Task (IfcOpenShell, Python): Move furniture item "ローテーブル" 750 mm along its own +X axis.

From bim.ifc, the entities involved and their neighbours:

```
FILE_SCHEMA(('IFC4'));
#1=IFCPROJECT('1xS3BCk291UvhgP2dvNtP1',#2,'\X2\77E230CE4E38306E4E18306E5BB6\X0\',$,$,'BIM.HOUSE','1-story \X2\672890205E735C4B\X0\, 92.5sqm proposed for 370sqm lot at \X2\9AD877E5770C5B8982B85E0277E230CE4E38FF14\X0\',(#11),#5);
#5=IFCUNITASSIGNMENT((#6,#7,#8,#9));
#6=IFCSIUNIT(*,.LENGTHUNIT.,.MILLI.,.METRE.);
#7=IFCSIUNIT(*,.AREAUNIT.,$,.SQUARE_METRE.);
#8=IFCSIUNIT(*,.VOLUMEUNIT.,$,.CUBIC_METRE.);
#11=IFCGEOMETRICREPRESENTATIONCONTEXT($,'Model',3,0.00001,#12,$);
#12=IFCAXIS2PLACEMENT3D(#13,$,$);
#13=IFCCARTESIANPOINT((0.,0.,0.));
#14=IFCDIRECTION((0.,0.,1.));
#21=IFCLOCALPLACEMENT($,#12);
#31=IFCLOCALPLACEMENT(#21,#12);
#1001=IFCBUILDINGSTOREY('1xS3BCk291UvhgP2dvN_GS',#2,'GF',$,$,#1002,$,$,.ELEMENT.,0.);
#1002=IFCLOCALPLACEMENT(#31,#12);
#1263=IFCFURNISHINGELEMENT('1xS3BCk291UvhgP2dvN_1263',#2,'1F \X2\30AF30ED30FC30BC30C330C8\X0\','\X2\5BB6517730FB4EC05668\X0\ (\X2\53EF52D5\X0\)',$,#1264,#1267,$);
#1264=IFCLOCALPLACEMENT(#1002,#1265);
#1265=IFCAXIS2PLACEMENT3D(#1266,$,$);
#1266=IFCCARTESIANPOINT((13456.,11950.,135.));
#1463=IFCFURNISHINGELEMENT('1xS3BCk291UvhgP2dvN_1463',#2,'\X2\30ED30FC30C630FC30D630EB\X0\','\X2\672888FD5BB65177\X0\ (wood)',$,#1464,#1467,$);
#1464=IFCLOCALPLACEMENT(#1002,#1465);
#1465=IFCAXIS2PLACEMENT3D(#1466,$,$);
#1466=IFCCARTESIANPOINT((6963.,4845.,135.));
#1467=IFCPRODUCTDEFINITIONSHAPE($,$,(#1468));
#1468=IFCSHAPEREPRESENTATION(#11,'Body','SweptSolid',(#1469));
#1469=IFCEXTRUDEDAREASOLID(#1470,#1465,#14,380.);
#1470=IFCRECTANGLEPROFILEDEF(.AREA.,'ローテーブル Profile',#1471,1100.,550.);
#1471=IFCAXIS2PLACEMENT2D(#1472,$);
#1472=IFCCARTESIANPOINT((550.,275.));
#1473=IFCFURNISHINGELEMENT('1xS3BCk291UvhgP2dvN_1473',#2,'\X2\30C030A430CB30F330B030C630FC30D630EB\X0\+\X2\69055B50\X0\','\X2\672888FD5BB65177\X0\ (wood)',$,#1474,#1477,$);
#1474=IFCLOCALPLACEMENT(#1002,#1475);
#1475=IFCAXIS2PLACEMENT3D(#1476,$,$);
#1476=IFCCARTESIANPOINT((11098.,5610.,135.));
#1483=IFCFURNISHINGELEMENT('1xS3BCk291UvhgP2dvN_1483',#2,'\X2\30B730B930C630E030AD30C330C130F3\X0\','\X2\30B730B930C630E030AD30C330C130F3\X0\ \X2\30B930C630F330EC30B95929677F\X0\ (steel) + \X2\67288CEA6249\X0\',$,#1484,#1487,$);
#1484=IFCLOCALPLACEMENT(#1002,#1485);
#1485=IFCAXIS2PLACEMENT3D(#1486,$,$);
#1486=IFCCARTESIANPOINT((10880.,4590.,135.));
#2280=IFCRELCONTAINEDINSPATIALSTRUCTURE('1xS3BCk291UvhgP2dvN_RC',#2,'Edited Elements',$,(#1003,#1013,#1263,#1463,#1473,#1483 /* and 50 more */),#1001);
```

```python
import ifcopenshell
import ifcopenshell.api.geometry
import ifcopenshell.util.placement

model = ifcopenshell.open("bim.ifc")

item = model.by_guid("1xS3BCk291UvhgP2dvN_1463")
matrix = ifcopenshell.util.placement.get_local_placement(item.ObjectPlacement)
matrix[:3, 3] += matrix[:3, 0] * 750.0
ifcopenshell.api.geometry.edit_object_placement(model, product=item, matrix=matrix, is_si=False)

print(ifcopenshell.util.placement.get_local_placement(item.ObjectPlacement).round(3) + 0.0)

model.write("bim_edited.ifc")
```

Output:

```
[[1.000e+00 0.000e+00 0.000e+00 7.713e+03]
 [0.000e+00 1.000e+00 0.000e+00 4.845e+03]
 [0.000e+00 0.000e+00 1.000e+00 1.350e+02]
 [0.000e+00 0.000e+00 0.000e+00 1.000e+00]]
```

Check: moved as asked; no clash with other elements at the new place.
